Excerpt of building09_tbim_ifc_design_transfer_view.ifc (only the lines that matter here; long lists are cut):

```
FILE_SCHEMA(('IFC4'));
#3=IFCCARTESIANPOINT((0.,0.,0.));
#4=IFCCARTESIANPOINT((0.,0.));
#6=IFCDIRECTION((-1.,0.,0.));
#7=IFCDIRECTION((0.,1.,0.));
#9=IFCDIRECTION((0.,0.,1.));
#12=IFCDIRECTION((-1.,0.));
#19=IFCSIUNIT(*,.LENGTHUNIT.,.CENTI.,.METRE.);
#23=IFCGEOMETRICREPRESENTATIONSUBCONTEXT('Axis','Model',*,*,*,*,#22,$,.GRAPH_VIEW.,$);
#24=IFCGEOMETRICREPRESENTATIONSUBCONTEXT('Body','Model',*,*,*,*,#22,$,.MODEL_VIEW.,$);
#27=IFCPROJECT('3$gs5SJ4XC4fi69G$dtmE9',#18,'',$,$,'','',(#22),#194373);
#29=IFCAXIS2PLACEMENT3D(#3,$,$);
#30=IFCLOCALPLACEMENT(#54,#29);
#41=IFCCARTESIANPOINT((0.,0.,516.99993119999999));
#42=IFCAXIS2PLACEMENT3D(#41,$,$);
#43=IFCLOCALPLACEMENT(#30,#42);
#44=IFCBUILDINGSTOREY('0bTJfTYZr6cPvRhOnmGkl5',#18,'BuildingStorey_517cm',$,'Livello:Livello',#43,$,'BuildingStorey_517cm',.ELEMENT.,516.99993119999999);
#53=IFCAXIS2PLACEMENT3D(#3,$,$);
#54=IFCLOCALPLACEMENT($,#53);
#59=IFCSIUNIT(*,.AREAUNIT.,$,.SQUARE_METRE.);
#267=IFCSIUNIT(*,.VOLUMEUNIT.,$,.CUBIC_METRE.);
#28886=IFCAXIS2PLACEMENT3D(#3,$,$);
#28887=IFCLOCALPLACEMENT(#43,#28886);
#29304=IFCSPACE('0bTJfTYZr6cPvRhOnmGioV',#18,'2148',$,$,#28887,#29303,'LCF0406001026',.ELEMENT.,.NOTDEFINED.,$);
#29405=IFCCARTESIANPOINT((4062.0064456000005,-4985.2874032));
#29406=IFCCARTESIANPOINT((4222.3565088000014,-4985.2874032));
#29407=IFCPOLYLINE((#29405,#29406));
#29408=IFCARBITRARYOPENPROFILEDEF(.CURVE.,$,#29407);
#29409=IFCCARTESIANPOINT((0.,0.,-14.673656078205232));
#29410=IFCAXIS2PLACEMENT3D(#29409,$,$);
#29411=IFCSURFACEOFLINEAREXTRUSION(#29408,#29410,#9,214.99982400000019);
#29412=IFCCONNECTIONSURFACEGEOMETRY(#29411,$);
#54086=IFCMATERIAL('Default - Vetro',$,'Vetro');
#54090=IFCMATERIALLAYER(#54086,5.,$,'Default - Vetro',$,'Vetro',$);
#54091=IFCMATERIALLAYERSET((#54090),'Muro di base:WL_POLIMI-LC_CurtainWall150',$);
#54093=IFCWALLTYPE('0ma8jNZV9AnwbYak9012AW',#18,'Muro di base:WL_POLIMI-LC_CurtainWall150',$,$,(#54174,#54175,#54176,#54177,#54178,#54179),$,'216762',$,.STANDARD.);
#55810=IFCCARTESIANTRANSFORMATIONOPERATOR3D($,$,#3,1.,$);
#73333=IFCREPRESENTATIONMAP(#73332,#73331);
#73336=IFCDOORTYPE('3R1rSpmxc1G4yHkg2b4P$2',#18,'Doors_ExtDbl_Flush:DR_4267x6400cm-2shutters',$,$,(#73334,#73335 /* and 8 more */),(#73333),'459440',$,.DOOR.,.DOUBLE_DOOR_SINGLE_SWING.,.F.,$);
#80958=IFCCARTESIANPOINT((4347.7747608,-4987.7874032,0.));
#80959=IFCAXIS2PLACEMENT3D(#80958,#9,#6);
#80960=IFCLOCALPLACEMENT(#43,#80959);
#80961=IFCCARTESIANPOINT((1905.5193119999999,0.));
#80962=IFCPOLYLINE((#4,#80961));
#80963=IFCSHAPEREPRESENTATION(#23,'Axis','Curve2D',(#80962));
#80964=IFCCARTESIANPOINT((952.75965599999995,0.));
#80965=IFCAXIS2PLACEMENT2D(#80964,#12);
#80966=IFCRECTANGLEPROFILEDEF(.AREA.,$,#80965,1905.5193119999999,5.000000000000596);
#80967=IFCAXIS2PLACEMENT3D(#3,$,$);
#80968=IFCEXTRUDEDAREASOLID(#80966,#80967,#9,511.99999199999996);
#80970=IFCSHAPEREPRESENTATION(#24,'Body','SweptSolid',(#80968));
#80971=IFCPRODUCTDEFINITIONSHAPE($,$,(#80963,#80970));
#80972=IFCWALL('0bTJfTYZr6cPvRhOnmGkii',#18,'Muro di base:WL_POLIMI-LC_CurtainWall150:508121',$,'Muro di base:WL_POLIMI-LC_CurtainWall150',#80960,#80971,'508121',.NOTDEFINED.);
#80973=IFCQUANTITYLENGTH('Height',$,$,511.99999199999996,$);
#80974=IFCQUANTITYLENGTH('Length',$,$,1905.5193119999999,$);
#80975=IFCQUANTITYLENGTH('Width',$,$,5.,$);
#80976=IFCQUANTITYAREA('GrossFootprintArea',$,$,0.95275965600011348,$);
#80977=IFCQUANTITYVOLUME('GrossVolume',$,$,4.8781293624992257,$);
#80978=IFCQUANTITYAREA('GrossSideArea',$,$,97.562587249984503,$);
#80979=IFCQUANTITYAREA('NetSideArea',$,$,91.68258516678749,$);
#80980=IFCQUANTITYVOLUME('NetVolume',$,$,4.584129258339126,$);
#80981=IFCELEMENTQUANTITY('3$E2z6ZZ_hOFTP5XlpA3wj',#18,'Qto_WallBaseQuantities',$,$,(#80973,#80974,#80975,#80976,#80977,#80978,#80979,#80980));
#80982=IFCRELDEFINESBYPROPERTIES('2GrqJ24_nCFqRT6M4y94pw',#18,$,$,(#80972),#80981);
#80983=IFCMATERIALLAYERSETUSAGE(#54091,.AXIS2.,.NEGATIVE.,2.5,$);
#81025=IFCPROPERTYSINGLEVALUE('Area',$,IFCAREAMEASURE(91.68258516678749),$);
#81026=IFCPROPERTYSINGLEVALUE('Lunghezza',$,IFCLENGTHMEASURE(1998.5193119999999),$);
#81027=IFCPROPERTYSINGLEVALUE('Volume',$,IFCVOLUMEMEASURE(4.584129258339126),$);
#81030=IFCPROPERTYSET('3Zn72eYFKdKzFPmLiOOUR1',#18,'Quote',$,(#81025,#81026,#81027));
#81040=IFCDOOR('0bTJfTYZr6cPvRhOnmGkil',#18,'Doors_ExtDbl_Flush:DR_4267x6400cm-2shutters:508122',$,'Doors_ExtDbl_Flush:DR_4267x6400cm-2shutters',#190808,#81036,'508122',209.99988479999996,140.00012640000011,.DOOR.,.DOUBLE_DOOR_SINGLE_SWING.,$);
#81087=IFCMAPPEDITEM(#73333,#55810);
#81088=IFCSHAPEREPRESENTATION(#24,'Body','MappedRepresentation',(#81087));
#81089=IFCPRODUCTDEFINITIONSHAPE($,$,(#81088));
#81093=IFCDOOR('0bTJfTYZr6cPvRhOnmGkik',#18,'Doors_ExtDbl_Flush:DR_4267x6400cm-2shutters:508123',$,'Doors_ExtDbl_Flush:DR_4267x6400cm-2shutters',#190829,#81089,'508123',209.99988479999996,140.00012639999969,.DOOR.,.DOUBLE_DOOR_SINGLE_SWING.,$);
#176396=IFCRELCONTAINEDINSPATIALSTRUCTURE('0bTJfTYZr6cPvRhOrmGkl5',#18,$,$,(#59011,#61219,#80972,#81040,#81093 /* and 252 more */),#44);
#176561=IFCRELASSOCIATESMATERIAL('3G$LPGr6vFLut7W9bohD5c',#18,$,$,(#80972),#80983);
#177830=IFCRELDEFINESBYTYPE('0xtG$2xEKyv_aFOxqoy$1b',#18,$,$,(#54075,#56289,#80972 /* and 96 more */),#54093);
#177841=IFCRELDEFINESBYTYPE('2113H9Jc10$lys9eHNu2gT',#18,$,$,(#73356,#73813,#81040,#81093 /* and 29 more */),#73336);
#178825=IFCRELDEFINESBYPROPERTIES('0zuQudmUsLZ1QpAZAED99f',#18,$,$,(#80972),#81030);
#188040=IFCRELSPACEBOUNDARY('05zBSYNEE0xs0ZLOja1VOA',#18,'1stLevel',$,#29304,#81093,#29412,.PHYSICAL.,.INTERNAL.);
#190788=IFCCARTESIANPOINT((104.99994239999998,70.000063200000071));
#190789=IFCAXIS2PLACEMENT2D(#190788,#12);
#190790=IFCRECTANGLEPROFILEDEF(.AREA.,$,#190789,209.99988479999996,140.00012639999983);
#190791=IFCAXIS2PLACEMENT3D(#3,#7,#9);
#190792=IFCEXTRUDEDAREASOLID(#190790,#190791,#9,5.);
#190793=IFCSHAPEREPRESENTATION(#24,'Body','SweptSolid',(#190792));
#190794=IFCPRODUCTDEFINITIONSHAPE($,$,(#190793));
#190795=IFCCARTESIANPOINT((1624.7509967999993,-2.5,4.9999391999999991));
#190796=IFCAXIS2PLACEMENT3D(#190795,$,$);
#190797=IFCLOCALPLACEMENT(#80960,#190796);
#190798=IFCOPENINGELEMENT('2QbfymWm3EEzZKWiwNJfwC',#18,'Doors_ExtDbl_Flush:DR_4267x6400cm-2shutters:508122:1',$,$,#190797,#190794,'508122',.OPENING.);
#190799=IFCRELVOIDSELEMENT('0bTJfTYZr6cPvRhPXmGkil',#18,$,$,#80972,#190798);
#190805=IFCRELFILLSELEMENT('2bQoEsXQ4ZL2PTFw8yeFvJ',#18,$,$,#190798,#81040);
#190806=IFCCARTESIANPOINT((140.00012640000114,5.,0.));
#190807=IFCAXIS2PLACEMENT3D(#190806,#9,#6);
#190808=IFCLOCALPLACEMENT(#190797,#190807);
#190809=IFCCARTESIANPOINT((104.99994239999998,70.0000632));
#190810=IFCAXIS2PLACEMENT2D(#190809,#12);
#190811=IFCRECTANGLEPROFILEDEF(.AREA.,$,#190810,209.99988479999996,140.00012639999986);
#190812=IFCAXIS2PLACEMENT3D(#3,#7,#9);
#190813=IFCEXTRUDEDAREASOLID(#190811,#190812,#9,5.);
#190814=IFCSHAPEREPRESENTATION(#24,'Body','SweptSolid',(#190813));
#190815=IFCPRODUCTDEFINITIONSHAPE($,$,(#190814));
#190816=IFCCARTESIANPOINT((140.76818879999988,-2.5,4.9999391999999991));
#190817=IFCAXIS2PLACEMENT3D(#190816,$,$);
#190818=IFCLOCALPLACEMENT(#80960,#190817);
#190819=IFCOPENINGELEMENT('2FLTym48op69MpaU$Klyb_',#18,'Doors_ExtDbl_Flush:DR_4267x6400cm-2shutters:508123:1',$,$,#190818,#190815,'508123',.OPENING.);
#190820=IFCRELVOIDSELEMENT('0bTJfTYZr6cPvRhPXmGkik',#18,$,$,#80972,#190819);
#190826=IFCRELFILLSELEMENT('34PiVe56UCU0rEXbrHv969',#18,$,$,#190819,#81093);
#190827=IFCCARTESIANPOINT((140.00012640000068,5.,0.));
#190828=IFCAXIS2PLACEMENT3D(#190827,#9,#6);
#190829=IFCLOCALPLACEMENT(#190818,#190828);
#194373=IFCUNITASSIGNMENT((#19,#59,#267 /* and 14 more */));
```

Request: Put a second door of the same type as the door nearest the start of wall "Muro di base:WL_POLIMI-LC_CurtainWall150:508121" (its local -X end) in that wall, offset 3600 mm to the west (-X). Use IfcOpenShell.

```python
import numpy as np
import ifcopenshell
import ifcopenshell.api.feature
import ifcopenshell.api.geometry
import ifcopenshell.api.pset
import ifcopenshell.api.root
import ifcopenshell.geom
import ifcopenshell.util.element
import ifcopenshell.util.placement
import ifcopenshell.util.shape
import ifcopenshell.util.unit

model = ifcopenshell.open("building09_tbim_ifc_design_transfer_view.ifc")
unit_scale = ifcopenshell.util.unit.calculate_unit_scale(model)
area_scale = ifcopenshell.util.unit.calculate_unit_scale(model, "AREAUNIT")
volume_scale = ifcopenshell.util.unit.calculate_unit_scale(model, "VOLUMEUNIT")
settings = ifcopenshell.geom.settings()


def volume(element):
    """Net volume in cubic metres, openings subtracted."""
    shape = ifcopenshell.geom.create_shape(settings, element)
    return ifcopenshell.util.shape.get_volume(shape.geometry)


def reuse_history(source, copy):
    """copy_class also copies each property set's owner history, people and application; keep the originals."""
    for rel in copy.IsDefinedBy:
        if rel.is_a("IfcRelDefinesByProperties") and (history := rel.RelatingPropertyDefinition.OwnerHistory):
            rel.RelatingPropertyDefinition.OwnerHistory = source.OwnerHistory
            ifcopenshell.util.element.remove_deep2(model, history)


door = model.by_id(81093)
opening = door.FillsVoids[0].RelatingOpeningElement
wall = opening.VoidsElements[0].RelatingBuildingElement
before = volume(wall)
shift = ifcopenshell.util.placement.get_local_placement(wall.ObjectPlacement)[:3, 0] * 3.6 / unit_scale

# copy_class copies the void relationship, type, container and properties, but no geometry.
new_opening = ifcopenshell.api.root.copy_class(model, product=opening)
new_opening.Representation = ifcopenshell.util.element.copy_deep(
    model, opening.Representation, exclude=["IfcGeometricRepresentationContext", "IfcRepresentationMap"]
)
new_opening.Name = "Doors_ExtDbl_Flush:DR_4267x6400cm-2shutters"
new_opening.Tag = None
reuse_history(opening, new_opening)
new_door = ifcopenshell.api.root.copy_class(model, product=door)
new_door.Representation = ifcopenshell.util.element.copy_deep(
    model, door.Representation, exclude=["IfcGeometricRepresentationContext", "IfcRepresentationMap"]
)
new_door.Name = "Doors_ExtDbl_Flush:DR_4267x6400cm-2shutters"
new_door.Tag = None
reuse_history(door, new_door)
ifcopenshell.api.feature.add_filling(model, opening=new_opening, element=new_door)

for old, new in ((opening, new_opening), (door, new_door)):
    matrix = ifcopenshell.util.placement.get_local_placement(old.ObjectPlacement)
    matrix[:3, 3] += shift
    ifcopenshell.api.geometry.edit_object_placement(model, product=new, matrix=matrix, is_si=False)

# The copied space boundaries still share their surfaces with the original.
for rel in new_door.ProvidesBoundaries:
    if rel.ConnectionGeometry:
        rel.ConnectionGeometry = ifcopenshell.util.element.copy_deep(model, rel.ConnectionGeometry)

# Space boundary surfaces are stored in each space's coordinates; move them too.
for rel in new_door.ProvidesBoundaries:
    if not rel.ConnectionGeometry:
        continue
    surface = rel.ConnectionGeometry.SurfaceOnRelatingElement
    space_matrix = ifcopenshell.util.placement.get_local_placement(rel.RelatingSpace.ObjectPlacement)
    point = np.array(surface.Position.Location.Coordinates) + space_matrix[:3, :3].T @ shift
    surface.Position = model.createIfcAxis2Placement3D(
        model.createIfcCartesianPoint(point.tolist()), surface.Position.Axis, surface.Position.RefDirection
    )

after = volume(wall)
thickness = 0.05  # wall thickness in metres

# Update the wall's stored quantities.
qto = model.by_id(ifcopenshell.util.element.get_pset(wall, "Qto_WallBaseQuantities", should_inherit=False)["id"])
ifcopenshell.api.pset.edit_qto(model, qto=qto, properties={
    "NetSideArea": after / thickness / area_scale,
    "NetVolume": after / volume_scale,
})
pset = model.by_id(ifcopenshell.util.element.get_pset(wall, "Quote", should_inherit=False)["id"])
ifcopenshell.api.pset.edit_pset(model, pset=pset, properties={
    "Area": model.create_entity("IfcAreaMeasure", after / thickness / area_scale),
    "Volume": model.create_entity("IfcVolumeMeasure", after / volume_scale),
})

print(f"wall volume {before:.3f} -> {after:.3f} m3")

model.write("building09_tbim_ifc_design_transfer_view_rev.ifc")
```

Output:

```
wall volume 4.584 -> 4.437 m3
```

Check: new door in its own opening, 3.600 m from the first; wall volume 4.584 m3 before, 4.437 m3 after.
